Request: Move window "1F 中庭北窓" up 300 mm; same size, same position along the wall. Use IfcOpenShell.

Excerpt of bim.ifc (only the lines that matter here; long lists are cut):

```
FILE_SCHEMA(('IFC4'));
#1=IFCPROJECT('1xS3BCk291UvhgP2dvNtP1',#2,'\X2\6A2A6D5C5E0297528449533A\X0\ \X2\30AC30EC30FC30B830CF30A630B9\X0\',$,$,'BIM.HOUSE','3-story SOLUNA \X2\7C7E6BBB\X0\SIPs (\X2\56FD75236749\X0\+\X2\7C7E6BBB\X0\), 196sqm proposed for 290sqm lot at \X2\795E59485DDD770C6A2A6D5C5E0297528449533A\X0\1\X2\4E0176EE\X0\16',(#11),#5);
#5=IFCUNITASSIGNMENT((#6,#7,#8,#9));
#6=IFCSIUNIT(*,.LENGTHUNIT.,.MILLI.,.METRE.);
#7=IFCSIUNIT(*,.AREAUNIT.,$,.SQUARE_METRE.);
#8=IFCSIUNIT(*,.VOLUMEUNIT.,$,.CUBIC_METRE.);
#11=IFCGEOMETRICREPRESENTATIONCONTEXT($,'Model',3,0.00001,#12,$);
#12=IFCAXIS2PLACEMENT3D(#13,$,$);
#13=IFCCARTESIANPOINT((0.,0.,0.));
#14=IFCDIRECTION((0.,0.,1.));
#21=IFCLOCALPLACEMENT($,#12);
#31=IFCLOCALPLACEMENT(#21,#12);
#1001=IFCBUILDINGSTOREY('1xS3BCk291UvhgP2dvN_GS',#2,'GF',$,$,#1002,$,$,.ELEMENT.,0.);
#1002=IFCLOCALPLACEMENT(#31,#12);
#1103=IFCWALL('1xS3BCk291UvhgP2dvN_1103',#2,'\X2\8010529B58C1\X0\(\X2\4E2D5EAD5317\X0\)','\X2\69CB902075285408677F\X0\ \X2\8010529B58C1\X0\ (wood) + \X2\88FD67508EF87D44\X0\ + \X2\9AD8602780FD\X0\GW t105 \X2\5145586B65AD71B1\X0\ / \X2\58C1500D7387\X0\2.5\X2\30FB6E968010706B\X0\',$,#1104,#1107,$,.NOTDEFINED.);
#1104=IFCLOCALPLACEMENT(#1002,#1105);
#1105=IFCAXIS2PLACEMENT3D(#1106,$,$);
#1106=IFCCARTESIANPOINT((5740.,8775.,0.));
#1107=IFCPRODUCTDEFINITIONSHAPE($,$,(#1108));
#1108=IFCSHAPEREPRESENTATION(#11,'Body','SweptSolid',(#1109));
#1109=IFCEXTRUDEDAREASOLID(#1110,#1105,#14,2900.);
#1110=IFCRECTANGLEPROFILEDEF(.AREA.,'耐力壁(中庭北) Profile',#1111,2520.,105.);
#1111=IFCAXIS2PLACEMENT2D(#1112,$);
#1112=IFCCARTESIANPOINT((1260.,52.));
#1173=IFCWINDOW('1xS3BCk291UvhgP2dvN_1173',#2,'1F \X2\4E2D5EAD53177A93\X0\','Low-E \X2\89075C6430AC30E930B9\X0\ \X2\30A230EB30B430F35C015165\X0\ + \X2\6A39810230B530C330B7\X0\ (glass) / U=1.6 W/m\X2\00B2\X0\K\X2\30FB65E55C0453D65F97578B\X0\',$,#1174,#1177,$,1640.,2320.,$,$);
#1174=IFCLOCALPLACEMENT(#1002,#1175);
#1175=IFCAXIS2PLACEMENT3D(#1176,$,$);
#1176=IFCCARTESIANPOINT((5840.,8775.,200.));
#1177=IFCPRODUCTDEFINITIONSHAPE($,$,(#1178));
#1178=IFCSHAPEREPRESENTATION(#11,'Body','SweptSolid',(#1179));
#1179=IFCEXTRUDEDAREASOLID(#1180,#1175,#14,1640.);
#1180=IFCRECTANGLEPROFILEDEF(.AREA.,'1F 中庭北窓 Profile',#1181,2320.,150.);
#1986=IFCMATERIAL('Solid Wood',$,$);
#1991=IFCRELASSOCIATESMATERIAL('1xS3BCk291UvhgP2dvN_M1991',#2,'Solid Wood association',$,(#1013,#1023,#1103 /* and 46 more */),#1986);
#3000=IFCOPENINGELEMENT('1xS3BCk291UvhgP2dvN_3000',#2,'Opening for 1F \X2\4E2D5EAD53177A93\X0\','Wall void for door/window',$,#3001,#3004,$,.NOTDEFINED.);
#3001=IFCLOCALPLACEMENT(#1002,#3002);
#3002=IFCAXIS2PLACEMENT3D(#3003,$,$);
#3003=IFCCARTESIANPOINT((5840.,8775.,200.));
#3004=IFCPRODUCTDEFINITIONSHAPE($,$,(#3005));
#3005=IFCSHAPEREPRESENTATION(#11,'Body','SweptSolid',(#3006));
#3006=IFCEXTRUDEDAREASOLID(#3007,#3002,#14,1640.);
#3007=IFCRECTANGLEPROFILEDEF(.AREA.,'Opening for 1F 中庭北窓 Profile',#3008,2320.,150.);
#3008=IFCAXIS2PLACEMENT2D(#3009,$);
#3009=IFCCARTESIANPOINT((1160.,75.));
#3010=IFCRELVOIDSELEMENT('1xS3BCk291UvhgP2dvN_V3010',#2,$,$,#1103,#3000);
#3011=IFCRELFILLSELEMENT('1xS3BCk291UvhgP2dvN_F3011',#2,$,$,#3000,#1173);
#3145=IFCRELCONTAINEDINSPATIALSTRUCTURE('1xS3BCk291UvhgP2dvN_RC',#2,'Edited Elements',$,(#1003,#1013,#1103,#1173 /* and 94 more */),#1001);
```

```python
import numpy as np
import ifcopenshell
import ifcopenshell.api.geometry
import ifcopenshell.util.placement
import ifcopenshell.util.unit

model = ifcopenshell.open("bim.ifc")
unit_scale = ifcopenshell.util.unit.calculate_unit_scale(model)

window = model.by_guid("1xS3BCk291UvhgP2dvN_1173")
opening = window.FillsVoids[0].RelatingOpeningElement
dz = 0.3 / unit_scale

shift = np.array([0.0, 0.0, dz])
# The window is not placed relative to its opening, so move both.
for product in (opening, window):
    matrix = ifcopenshell.util.placement.get_local_placement(product.ObjectPlacement)
    matrix[:3, 3] += shift
    ifcopenshell.api.geometry.edit_object_placement(model, product=product, matrix=matrix, is_si=False)

print(f"moved by {dz * unit_scale:+.3f} m")

model.write("bim_rev.ifc")
```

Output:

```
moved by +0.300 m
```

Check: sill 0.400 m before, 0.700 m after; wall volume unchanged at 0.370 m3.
